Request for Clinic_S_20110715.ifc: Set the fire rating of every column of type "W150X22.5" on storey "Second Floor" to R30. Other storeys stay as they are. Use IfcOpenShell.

First a look at what the model holds.

```python
import ifcopenshell
import ifcopenshell.util.element

model = ifcopenshell.open("Clinic_S_20110715.ifc")
print(model.schema)
storey = next(s for s in model.by_type("IfcBuildingStorey") if s.Name == "Second Floor")
columns = [e for e in ifcopenshell.util.element.get_decomposition(storey) if e.is_a("IfcColumn")]
seen = {}
for e in columns:
    element_type = ifcopenshell.util.element.get_type(e)
    key = (element_type.Name if element_type != e and element_type else None, ifcopenshell.util.element.get_pset(e, "Pset_ColumnCommon", "FireRating"))
    seen[key] = seen.get(key, 0) + 1
for (name, value), count in sorted(seen.items(), key=str):
    print(count, "x", name, "|", value)
```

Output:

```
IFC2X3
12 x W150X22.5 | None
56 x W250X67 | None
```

```python
import ifcopenshell
import ifcopenshell.api.pset
import ifcopenshell.util.element

model = ifcopenshell.open("Clinic_S_20110715.ifc")

storey = next(s for s in model.by_type("IfcBuildingStorey") if s.Name == "Second Floor")
columns = [e for e in ifcopenshell.util.element.get_decomposition(storey) if e.is_a("IfcColumn")]

count = 0
for e in columns:
    element_type = ifcopenshell.util.element.get_type(e)
    if element_type in (None, e) or element_type.Name != "W150X22.5":
        continue
    # add_pset returns the element's existing set when there is one.
    pset = ifcopenshell.api.pset.add_pset(model, product=e, name="Pset_ColumnCommon")
    ifcopenshell.api.pset.edit_pset(model, pset=pset, properties={"FireRating": "R30"})
    count += 1

print(count, "columns updated")

model.write("Clinic_S_20110715_edited.ifc")
```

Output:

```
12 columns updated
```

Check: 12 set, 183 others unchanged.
